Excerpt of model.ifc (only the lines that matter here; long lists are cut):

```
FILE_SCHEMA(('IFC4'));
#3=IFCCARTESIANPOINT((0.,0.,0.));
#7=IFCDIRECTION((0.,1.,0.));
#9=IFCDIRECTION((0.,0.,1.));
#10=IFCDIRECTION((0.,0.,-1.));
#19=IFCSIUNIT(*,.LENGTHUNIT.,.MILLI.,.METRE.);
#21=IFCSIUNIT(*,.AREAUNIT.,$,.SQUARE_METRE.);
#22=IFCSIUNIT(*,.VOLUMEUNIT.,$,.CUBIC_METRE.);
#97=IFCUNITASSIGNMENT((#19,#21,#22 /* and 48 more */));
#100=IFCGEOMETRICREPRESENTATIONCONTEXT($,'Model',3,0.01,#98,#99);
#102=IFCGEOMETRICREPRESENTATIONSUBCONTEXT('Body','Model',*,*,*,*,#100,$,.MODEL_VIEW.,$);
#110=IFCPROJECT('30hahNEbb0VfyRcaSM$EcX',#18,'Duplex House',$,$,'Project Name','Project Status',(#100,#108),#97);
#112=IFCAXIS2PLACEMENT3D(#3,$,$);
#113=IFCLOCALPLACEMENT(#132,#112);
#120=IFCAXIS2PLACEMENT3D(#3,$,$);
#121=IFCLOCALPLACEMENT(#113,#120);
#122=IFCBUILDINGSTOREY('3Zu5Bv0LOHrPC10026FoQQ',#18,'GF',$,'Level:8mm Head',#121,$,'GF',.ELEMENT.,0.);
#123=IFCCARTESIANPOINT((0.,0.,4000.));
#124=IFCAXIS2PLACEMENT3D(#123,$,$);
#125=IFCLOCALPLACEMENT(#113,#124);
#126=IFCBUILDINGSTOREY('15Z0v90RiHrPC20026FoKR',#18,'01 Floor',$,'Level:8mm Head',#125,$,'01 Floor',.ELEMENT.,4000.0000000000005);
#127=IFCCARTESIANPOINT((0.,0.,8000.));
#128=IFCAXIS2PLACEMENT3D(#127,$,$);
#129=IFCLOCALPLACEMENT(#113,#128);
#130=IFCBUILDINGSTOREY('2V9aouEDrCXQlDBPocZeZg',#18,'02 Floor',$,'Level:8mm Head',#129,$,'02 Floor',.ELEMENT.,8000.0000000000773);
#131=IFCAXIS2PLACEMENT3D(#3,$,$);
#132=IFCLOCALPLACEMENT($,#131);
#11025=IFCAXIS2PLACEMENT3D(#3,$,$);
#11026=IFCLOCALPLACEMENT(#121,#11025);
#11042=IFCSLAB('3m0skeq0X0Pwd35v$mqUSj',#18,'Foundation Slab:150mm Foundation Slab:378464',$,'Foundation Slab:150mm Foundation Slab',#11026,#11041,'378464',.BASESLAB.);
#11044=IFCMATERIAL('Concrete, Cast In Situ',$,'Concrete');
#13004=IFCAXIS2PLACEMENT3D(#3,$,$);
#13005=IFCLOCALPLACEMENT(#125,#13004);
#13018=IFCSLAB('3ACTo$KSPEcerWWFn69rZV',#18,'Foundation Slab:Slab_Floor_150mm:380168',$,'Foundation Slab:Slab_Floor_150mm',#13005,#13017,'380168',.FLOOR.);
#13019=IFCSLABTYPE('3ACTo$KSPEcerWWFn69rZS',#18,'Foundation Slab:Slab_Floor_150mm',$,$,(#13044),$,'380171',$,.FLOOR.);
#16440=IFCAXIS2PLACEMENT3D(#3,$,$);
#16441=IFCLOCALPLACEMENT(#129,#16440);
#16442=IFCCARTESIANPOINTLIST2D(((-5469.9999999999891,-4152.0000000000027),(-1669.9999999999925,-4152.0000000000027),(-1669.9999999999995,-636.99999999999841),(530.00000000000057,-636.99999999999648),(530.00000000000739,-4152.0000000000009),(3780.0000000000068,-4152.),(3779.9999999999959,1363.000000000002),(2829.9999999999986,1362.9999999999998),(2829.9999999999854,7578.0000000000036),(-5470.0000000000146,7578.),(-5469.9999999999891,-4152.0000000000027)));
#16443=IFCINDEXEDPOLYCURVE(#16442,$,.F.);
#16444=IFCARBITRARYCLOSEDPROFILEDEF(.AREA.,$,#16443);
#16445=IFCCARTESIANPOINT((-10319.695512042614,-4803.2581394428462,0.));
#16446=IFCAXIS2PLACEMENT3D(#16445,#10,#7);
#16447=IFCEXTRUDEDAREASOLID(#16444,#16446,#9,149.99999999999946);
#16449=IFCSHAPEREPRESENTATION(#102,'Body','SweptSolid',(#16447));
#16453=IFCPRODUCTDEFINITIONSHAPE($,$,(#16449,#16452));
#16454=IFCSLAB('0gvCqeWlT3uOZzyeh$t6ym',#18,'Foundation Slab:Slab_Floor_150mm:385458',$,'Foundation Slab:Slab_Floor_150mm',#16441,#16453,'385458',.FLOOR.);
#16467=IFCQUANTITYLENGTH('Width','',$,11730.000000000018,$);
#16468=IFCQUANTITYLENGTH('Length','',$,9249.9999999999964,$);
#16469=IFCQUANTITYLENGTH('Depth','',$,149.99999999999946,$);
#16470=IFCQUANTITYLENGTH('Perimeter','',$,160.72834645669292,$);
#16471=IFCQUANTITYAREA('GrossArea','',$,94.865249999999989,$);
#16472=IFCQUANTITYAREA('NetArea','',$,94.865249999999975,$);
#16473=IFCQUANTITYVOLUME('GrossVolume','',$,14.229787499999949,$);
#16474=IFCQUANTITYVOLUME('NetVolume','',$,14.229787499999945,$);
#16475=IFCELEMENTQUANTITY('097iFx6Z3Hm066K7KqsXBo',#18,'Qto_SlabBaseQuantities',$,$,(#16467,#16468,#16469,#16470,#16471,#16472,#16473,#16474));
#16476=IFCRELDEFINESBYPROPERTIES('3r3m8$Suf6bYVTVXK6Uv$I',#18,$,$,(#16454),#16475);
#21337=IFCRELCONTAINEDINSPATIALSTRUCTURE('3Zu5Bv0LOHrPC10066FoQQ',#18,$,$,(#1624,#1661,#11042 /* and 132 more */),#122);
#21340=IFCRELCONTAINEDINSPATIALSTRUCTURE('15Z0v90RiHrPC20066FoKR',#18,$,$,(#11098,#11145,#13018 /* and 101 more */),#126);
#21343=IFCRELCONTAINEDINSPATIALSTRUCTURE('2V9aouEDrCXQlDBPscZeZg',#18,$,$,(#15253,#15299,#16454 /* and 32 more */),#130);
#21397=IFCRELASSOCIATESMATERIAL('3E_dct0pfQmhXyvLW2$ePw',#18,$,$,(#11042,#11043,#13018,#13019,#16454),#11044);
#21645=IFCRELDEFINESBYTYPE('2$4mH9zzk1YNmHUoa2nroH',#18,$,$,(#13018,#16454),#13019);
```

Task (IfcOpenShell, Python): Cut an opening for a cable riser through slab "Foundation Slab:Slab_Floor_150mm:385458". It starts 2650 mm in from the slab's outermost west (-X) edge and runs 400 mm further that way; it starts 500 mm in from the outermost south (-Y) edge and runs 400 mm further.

```python
import numpy as np
import ifcopenshell
import ifcopenshell.api.feature
import ifcopenshell.api.geometry
import ifcopenshell.api.pset
import ifcopenshell.api.root
import ifcopenshell.geom
import ifcopenshell.util.element
import ifcopenshell.util.placement
import ifcopenshell.util.representation
import ifcopenshell.util.shape
import ifcopenshell.util.unit

model = ifcopenshell.open("model.ifc")
unit_scale = ifcopenshell.util.unit.calculate_unit_scale(model)
area_scale = ifcopenshell.util.unit.calculate_unit_scale(model, "AREAUNIT")
volume_scale = ifcopenshell.util.unit.calculate_unit_scale(model, "VOLUMEUNIT")
settings = ifcopenshell.geom.settings()


def volume(element):
    """Net volume in cubic metres, openings subtracted."""
    shape = ifcopenshell.geom.create_shape(settings, element)
    return ifcopenshell.util.shape.get_volume(shape.geometry)


slab = model.by_guid("0gvCqeWlT3uOZzyeh$t6ym")
before = volume(slab)

# Extent in the slab's own axes, in metres. The edges named are its -X and -Y sides.
slab_shape = ifcopenshell.geom.create_shape(settings, slab)
vertices = ifcopenshell.util.shape.get_vertices(slab_shape.geometry)
x_min, y_min, bottom = vertices.min(axis=0)
top = vertices[:, 2].max()

opening = ifcopenshell.api.root.create_entity(model, ifc_class="IfcOpeningElement", name="Cable riser opening", predefined_type="OPENING")
context = ifcopenshell.util.representation.get_context(model, "Model", "Body", "MODEL_VIEW")
width, depth = 0.4, 0.4
outline = [(0.0, 0.0), (width, 0.0), (width, depth), (0.0, depth), (0.0, 0.0)]
# Overshoot both faces by 50 mm so the cut is clean.
shape = ifcopenshell.api.geometry.add_slab_representation(
    model, context=context, depth=top - bottom + 0.1, polyline=outline
)
ifcopenshell.api.geometry.assign_representation(model, product=opening, representation=shape)

matrix = ifcopenshell.util.placement.get_local_placement(slab.ObjectPlacement)
matrix[:, 3] = matrix @ np.append(np.array([x_min + 2.65, y_min + 0.5, bottom - 0.05]) / unit_scale, 1.0)
ifcopenshell.api.geometry.edit_object_placement(model, product=opening, matrix=matrix, is_si=False)
ifcopenshell.api.feature.add_feature(model, feature=opening, element=slab)

after = volume(slab)

# Update the slab's stored quantities.
qto = model.by_id(ifcopenshell.util.element.get_pset(slab, "Qto_SlabBaseQuantities", should_inherit=False)["id"])
ifcopenshell.api.pset.edit_qto(model, qto=qto, properties={
    "NetArea": after / (top - bottom) / area_scale,
    "NetVolume": after / volume_scale,
})

print(f"slab volume {before:.3f} -> {after:.3f} m3")

model.write("model-out.ifc")
```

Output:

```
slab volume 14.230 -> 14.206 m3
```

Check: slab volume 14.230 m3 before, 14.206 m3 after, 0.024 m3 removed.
